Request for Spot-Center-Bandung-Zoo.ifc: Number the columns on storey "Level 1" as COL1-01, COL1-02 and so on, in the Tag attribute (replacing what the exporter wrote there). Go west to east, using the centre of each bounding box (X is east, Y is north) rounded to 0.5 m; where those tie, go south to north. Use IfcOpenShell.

First a look at what the model holds.

```python
import ifcopenshell
import ifcopenshell.util.element
import ifcopenshell.util.placement

model = ifcopenshell.open("Spot-Center-Bandung-Zoo.ifc")
print(model.schema)
storey = next(s for s in model.by_type("IfcBuildingStorey") if s.Name == "Level 1")
columns = [e for e in ifcopenshell.util.element.get_decomposition(storey) if e.is_a("IfcColumn")]
for e in sorted(columns, key=lambda e: e.id()):
    origin = ifcopenshell.util.placement.get_local_placement(e.ObjectPlacement)[:3, 3]
    print(e.id(), e.Tag, e.Name, origin.round(2) + 0.0, sep=" | ")
```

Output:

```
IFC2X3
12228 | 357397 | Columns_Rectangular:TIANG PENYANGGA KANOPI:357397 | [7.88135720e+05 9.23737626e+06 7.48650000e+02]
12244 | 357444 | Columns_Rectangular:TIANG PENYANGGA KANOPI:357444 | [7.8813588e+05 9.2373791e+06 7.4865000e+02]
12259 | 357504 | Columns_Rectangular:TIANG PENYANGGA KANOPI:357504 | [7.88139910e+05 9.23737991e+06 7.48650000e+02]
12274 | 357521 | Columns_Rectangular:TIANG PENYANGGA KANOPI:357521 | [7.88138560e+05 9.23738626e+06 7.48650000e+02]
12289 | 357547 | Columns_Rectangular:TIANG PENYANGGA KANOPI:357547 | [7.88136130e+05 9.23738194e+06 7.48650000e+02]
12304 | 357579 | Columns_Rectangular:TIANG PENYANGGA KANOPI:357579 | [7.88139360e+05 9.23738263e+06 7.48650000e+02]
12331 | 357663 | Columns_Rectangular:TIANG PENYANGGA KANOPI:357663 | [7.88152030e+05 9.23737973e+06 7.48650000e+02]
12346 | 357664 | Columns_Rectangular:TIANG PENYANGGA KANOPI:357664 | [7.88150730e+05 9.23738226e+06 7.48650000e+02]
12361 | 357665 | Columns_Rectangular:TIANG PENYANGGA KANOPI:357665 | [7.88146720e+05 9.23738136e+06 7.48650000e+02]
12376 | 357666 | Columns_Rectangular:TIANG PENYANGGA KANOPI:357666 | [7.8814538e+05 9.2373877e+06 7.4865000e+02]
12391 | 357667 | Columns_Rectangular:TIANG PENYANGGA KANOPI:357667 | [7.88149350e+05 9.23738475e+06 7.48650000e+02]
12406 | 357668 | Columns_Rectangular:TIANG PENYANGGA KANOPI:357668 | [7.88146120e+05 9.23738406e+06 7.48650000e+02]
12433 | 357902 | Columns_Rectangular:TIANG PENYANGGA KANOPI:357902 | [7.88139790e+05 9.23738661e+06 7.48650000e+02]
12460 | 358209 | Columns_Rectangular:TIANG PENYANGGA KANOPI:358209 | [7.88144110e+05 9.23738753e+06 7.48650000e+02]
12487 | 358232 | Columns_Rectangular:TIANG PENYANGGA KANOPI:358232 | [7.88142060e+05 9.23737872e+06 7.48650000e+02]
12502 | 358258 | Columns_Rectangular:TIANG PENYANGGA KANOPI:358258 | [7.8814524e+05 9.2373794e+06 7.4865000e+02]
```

```python
import ifcopenshell
import ifcopenshell.geom
import ifcopenshell.util.element
import ifcopenshell.util.shape

model = ifcopenshell.open("Spot-Center-Bandung-Zoo.ifc")
settings = ifcopenshell.geom.settings()
settings.set("use-world-coords", True)


def centre(element):
    shape = ifcopenshell.geom.create_shape(settings, element)
    return ifcopenshell.util.shape.get_bbox_centroid(shape.geometry)


storey = next(s for s in model.by_type("IfcBuildingStorey") if s.Name == "Level 1")
columns = [e for e in ifcopenshell.util.element.get_decomposition(storey) if e.is_a("IfcColumn")]

# Insertion points can sit at a corner or the storey origin, so sort by the geometry (in metres).
centres = {e: centre(e) for e in columns}
columns.sort(key=lambda e: (round(centres[e][0] / 0.5), centres[e][1]))

for i, e in enumerate(columns, start=1):
    number = f"COL1-{i:02d}"
    e.Tag = number
    print(e.id(), number)

model.write("Spot-Center-Bandung-Zoo_edited.ifc")
```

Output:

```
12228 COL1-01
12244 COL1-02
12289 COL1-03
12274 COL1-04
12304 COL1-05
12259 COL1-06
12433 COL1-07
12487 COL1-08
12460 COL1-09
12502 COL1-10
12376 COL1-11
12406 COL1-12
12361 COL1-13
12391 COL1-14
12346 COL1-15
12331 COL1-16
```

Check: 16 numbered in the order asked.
